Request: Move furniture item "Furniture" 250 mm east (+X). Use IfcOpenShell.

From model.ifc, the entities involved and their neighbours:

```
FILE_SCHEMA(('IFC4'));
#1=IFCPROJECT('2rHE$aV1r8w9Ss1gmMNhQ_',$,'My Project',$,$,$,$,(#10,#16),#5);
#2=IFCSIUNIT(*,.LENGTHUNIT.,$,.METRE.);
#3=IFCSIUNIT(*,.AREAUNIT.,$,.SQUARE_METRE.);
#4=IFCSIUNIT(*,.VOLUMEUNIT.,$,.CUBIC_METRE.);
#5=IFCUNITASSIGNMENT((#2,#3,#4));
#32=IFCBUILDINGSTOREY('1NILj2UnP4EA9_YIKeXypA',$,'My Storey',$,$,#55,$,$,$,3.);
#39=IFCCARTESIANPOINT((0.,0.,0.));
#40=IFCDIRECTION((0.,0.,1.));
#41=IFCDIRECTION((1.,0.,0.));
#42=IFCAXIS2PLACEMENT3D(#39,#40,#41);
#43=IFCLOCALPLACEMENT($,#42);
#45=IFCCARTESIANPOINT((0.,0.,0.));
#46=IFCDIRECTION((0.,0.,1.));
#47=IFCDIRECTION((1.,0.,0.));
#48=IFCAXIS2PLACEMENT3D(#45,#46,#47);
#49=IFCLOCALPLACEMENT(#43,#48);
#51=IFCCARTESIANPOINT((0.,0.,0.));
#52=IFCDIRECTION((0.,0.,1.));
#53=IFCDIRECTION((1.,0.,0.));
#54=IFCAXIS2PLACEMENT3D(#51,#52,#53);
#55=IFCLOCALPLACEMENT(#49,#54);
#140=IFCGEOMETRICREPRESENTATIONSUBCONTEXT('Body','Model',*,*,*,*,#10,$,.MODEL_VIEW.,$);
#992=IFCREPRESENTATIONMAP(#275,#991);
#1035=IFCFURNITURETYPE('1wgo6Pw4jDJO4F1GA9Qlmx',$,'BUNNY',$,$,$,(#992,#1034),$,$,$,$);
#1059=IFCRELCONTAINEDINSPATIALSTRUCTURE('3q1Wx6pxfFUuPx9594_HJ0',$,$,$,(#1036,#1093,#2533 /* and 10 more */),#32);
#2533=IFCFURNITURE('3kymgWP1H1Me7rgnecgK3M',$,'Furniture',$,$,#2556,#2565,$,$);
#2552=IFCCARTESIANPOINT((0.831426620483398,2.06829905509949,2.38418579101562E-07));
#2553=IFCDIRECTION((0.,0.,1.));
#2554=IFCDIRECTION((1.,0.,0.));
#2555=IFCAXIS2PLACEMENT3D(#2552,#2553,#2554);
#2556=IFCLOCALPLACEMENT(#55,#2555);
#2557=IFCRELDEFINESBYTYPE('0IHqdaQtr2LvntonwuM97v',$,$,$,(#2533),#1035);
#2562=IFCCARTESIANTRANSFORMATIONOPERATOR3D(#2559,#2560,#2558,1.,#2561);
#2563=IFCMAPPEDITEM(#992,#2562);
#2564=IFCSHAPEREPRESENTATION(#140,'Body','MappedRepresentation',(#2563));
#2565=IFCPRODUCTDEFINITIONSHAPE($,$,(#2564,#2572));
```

```python
import ifcopenshell
import ifcopenshell.api.geometry
import ifcopenshell.util.placement
import ifcopenshell.util.unit

model = ifcopenshell.open("model.ifc")
unit_scale = ifcopenshell.util.unit.calculate_unit_scale(model)

item = model.by_id(2533)
matrix = ifcopenshell.util.placement.get_local_placement(item.ObjectPlacement)
matrix[0, 3] += 0.25 / unit_scale
ifcopenshell.api.geometry.edit_object_placement(model, product=item, matrix=matrix, is_si=False)

print(ifcopenshell.util.placement.get_local_placement(item.ObjectPlacement).round(3) + 0.0)

model.write("model_updated.ifc")
```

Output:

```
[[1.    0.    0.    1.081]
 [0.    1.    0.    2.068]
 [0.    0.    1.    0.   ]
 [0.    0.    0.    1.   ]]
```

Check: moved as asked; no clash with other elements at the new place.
